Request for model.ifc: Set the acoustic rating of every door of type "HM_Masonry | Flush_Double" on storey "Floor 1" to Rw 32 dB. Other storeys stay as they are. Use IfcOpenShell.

First a look at what the model holds.

```python
import ifcopenshell
import ifcopenshell.util.element

model = ifcopenshell.open("model.ifc")
print(model.schema)
storey = next(s for s in model.by_type("IfcBuildingStorey") if s.Name == "Floor 1")
doors = [e for e in ifcopenshell.util.element.get_decomposition(storey) if e.is_a("IfcDoor")]
seen = {}
for e in doors:
    element_type = ifcopenshell.util.element.get_type(e)
    key = (element_type.Name if element_type != e and element_type else None, ifcopenshell.util.element.get_pset(e, "Pset_DoorCommon", "AcousticRating"))
    seen[key] = seen.get(key, 0) + 1
for (name, value), count in sorted(seen.items(), key=str):
    print(count, "x", name, "|", value)
```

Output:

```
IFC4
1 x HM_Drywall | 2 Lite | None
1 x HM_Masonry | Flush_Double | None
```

```python
import ifcopenshell
import ifcopenshell.api.pset
import ifcopenshell.util.element

model = ifcopenshell.open("model.ifc")

storey = next(s for s in model.by_type("IfcBuildingStorey") if s.Name == "Floor 1")
doors = [e for e in ifcopenshell.util.element.get_decomposition(storey) if e.is_a("IfcDoor")]

count = 0
for e in doors:
    element_type = ifcopenshell.util.element.get_type(e)
    if element_type in (None, e) or element_type.Name != "HM_Masonry | Flush_Double":
        continue
    # add_pset returns the element's existing set when there is one.
    pset = ifcopenshell.api.pset.add_pset(model, product=e, name="Pset_DoorCommon")
    ifcopenshell.api.pset.edit_pset(model, pset=pset, properties={"AcousticRating": "Rw 32 dB"})
    count += 1

print(count, "doors updated")

model.write("model-out.ifc")
```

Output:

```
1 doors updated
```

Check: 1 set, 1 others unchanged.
